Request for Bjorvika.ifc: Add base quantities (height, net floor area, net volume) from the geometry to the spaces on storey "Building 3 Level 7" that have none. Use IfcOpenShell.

First a look at what the model holds.

```python
import ifcopenshell
import ifcopenshell.util.element
import ifcopenshell.util.unit

model = ifcopenshell.open("Bjorvika.ifc")
print(model.schema)
for unit_type in ("LENGTHUNIT", "AREAUNIT", "VOLUMEUNIT"):
    print(unit_type, ifcopenshell.util.unit.calculate_unit_scale(model, unit_type))
storey = next(s for s in model.by_type("IfcBuildingStorey") if s.Name == "Building 3 Level 7")
spaces = [e for e in ifcopenshell.util.element.get_decomposition(storey) if e.is_a("IfcSpace")]
for e in sorted(spaces, key=lambda e: e.id()):
    print(e.id(), e.is_a(), e.Name, list(ifcopenshell.util.element.get_psets(e, qtos_only=True)), sep=" | ")
```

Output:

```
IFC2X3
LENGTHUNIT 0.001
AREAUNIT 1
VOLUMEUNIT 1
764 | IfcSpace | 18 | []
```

```python
import ifcopenshell
import ifcopenshell.api.pset
import ifcopenshell.geom
import ifcopenshell.util.element
import ifcopenshell.util.shape
import ifcopenshell.util.unit

model = ifcopenshell.open("Bjorvika.ifc")
unit_scale = ifcopenshell.util.unit.calculate_unit_scale(model)
area_scale = ifcopenshell.util.unit.calculate_unit_scale(model, "AREAUNIT")
volume_scale = ifcopenshell.util.unit.calculate_unit_scale(model, "VOLUMEUNIT")
settings = ifcopenshell.geom.settings()

storey = next(s for s in model.by_type("IfcBuildingStorey") if s.Name == "Building 3 Level 7")
spaces = [e for e in ifcopenshell.util.element.get_decomposition(storey) if e.is_a("IfcSpace")]

for e in sorted(spaces, key=lambda e: e.id()):
    if ifcopenshell.util.element.get_psets(e, qtos_only=True, should_inherit=False):
        continue
    # Geometry comes back in metres, in the element's own axes.
    shape = ifcopenshell.geom.create_shape(settings, e)
    values = {
        "Height": ifcopenshell.util.shape.get_z(shape.geometry) / unit_scale,
        "NetFloorArea": ifcopenshell.util.shape.get_footprint_area(shape.geometry) / area_scale,
        "NetVolume": ifcopenshell.util.shape.get_volume(shape.geometry) / volume_scale,
    }
    qto = ifcopenshell.api.pset.add_qto(model, product=e, name="BaseQuantities")
    ifcopenshell.api.pset.edit_qto(model, qto=qto, properties=values)
    print(e.id(), {k: round(v, 3) for k, v in values.items()})

model.write("Bjorvika_rev.ifc")
```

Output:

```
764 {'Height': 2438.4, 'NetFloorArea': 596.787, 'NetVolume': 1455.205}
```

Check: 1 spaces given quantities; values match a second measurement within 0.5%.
